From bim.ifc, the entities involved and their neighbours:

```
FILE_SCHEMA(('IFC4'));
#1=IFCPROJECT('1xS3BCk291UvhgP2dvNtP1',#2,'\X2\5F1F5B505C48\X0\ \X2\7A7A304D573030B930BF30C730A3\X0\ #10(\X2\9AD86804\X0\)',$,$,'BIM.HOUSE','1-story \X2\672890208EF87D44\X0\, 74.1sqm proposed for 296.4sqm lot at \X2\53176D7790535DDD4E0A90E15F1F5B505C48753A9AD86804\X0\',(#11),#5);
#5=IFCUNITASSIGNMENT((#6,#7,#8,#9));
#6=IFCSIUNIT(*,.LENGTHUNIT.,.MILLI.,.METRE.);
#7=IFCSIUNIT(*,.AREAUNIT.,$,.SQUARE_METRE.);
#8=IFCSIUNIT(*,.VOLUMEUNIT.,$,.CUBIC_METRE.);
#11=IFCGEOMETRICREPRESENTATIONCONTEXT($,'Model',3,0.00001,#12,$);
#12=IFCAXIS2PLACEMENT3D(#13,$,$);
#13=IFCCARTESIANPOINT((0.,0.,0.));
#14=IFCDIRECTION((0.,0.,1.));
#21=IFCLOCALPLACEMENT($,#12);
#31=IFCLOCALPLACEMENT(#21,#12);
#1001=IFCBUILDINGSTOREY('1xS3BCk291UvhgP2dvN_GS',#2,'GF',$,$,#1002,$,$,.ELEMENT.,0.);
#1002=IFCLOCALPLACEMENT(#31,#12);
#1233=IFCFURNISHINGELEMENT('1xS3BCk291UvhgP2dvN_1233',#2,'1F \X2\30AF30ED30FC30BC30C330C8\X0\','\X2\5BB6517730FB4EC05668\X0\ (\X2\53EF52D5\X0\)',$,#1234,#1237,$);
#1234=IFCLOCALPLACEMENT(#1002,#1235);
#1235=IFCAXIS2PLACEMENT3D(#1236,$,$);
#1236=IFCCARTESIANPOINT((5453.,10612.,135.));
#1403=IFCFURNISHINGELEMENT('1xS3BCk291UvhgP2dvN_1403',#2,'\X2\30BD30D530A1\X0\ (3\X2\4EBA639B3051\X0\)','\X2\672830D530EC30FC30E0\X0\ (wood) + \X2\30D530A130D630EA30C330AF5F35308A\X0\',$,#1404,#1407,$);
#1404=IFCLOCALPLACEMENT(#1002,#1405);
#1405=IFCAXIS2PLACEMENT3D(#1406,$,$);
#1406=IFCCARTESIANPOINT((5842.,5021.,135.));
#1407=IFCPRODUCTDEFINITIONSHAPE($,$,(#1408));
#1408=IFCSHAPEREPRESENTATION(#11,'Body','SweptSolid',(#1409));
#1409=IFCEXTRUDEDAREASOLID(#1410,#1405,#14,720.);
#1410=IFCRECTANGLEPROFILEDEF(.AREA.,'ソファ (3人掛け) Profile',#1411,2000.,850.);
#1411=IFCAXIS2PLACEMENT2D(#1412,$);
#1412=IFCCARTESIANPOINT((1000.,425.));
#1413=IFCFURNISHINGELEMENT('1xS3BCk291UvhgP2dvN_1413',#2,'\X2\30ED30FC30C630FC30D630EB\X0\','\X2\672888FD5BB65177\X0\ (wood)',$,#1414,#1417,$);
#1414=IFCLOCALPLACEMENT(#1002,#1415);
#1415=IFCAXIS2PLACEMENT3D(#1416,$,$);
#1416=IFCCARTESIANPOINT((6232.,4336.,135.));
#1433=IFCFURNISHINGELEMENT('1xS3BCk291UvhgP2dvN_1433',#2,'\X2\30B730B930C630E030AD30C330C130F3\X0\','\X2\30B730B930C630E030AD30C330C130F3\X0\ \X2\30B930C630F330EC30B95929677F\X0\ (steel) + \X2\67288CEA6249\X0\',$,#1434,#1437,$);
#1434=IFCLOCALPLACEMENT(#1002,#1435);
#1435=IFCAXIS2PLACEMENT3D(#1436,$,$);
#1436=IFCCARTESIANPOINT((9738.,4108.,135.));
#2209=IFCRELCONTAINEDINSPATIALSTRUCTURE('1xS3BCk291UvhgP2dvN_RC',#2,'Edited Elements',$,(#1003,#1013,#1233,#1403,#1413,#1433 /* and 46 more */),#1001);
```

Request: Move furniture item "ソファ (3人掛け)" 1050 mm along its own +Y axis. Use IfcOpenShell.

```python
import ifcopenshell
import ifcopenshell.api.geometry
import ifcopenshell.util.placement
import ifcopenshell.util.unit

model = ifcopenshell.open("bim.ifc")
unit_scale = ifcopenshell.util.unit.calculate_unit_scale(model)

item = model.by_guid("1xS3BCk291UvhgP2dvN_1403")
matrix = ifcopenshell.util.placement.get_local_placement(item.ObjectPlacement)
matrix[:3, 3] += matrix[:3, 1] * 1.05 / unit_scale
ifcopenshell.api.geometry.edit_object_placement(model, product=item, matrix=matrix, is_si=False)

print(ifcopenshell.util.placement.get_local_placement(item.ObjectPlacement).round(3) + 0.0)

model.write("bim-out.ifc")
```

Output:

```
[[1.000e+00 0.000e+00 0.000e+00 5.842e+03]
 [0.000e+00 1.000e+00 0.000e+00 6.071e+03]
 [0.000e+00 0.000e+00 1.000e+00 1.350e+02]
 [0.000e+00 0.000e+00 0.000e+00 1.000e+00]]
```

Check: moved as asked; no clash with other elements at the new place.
